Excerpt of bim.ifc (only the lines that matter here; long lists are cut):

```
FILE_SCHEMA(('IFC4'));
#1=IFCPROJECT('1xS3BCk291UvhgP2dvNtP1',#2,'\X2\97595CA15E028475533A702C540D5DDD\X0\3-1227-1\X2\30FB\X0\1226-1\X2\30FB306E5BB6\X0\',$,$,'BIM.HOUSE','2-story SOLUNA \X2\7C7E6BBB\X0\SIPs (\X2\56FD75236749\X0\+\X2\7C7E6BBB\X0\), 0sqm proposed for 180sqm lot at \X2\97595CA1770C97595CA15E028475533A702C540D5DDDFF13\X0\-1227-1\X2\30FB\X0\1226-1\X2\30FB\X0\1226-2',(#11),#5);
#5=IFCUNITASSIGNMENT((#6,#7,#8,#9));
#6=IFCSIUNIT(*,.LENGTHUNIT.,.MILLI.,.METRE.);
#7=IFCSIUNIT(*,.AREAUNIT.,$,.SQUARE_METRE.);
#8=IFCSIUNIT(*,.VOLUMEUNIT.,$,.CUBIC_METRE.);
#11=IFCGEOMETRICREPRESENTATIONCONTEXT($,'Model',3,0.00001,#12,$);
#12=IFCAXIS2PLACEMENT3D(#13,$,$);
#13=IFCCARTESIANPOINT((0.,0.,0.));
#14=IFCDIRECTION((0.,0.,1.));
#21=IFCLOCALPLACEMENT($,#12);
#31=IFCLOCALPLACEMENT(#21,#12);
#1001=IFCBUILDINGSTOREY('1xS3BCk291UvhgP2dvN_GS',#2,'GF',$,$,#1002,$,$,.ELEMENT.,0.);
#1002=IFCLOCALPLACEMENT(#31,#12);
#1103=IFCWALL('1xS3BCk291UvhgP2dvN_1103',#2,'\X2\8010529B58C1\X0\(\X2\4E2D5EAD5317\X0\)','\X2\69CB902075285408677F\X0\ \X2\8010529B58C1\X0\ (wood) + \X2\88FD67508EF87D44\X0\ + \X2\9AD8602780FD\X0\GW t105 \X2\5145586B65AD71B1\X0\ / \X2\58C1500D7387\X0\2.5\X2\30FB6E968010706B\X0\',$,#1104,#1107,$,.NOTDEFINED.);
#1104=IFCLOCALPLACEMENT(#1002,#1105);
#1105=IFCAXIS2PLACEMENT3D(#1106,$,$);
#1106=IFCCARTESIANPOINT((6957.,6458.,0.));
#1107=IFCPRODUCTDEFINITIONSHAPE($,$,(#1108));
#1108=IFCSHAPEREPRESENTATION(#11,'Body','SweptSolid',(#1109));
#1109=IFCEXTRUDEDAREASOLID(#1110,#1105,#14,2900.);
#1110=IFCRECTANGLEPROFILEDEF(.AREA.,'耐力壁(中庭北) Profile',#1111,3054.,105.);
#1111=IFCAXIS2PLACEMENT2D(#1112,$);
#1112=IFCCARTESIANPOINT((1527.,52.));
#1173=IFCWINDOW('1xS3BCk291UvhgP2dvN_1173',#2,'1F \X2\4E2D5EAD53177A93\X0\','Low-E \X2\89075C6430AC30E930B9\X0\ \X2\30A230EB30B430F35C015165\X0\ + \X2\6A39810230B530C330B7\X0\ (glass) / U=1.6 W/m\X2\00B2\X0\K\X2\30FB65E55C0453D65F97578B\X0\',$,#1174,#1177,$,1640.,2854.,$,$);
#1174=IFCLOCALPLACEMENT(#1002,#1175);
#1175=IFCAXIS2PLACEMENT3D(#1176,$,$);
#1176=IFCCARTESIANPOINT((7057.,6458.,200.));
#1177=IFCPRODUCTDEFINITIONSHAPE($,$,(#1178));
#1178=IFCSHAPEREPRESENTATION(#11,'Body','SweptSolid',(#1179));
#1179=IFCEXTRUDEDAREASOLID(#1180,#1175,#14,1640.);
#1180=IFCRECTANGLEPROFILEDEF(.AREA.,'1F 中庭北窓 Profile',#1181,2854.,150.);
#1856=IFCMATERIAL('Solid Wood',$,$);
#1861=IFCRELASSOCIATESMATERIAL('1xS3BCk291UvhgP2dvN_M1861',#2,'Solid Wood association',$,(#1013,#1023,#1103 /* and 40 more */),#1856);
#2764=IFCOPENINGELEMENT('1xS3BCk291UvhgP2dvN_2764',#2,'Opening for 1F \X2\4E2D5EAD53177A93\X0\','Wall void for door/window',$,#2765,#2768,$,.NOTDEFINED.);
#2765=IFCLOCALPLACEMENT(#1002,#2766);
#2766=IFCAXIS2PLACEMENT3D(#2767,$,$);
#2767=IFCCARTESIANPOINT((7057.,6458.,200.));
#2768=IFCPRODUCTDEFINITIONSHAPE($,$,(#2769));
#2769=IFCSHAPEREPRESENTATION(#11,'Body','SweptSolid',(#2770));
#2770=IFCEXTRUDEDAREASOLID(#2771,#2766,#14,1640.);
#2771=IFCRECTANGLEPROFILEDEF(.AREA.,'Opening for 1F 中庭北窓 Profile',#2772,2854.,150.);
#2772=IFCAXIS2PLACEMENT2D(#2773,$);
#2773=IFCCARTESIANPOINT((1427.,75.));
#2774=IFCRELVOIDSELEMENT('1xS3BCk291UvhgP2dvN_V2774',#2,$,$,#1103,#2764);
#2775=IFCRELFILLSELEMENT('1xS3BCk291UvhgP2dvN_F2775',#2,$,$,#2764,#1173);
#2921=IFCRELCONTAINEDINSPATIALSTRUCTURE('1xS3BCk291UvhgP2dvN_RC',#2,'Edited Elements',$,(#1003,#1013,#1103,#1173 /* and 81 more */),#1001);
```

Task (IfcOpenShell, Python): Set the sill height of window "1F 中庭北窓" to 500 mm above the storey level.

```python
import numpy as np
import ifcopenshell
import ifcopenshell.api.geometry
import ifcopenshell.geom
import ifcopenshell.util.element
import ifcopenshell.util.placement
import ifcopenshell.util.shape
import ifcopenshell.util.unit

model = ifcopenshell.open("bim.ifc")
unit_scale = ifcopenshell.util.unit.calculate_unit_scale(model)

window = model.by_guid("1xS3BCk291UvhgP2dvN_1173")
opening = window.FillsVoids[0].RelatingOpeningElement
storey = ifcopenshell.util.element.get_container(window, ifc_class="IfcBuildingStorey")
level = ifcopenshell.util.placement.get_local_placement(storey.ObjectPlacement)[2, 3]

# The opening's origin need not be at the sill, so measure its lowest point.
shape = ifcopenshell.geom.create_shape(ifcopenshell.geom.settings(), opening)
bottom = ifcopenshell.util.shape.get_shape_bottom_elevation(shape, shape.geometry) / unit_scale
dz = level + 0.5 / unit_scale - bottom

shift = np.array([0.0, 0.0, dz])
# The window is not placed relative to its opening, so move both.
for product in (opening, window):
    matrix = ifcopenshell.util.placement.get_local_placement(product.ObjectPlacement)
    matrix[:3, 3] += shift
    ifcopenshell.api.geometry.edit_object_placement(model, product=product, matrix=matrix, is_si=False)

print(f"moved by {dz * unit_scale:+.3f} m")

model.write("bim_rev.ifc")
```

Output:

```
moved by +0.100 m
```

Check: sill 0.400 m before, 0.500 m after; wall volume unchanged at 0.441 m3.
